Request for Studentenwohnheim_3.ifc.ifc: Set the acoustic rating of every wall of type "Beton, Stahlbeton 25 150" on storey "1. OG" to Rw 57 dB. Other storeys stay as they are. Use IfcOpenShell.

First a look at what the model holds.

```python
import ifcopenshell
import ifcopenshell.util.element

model = ifcopenshell.open("Studentenwohnheim_3.ifc.ifc")
print(model.schema)
storey = next(s for s in model.by_type("IfcBuildingStorey") if s.Name == "1. OG")
walls = [e for e in ifcopenshell.util.element.get_decomposition(storey) if e.is_a("IfcWall")]
seen = {}
for e in walls:
    element_type = ifcopenshell.util.element.get_type(e)
    key = (element_type.Name if element_type != e and element_type else None, ifcopenshell.util.element.get_pset(e, "Pset_WallCommon", "AcousticRating"))
    seen[key] = seen.get(key, 0) + 1
for (name, value), count in sorted(seen.items(), key=str):
    print(count, "x", name, "|", value)
```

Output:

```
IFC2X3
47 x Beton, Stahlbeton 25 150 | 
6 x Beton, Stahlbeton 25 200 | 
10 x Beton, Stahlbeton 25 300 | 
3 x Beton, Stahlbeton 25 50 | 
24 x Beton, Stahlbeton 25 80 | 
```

```python
import ifcopenshell
import ifcopenshell.api.pset
import ifcopenshell.util.element

model = ifcopenshell.open("Studentenwohnheim_3.ifc.ifc")

storey = next(s for s in model.by_type("IfcBuildingStorey") if s.Name == "1. OG")
walls = [e for e in ifcopenshell.util.element.get_decomposition(storey) if e.is_a("IfcWall")]

count = 0
for e in walls:
    element_type = ifcopenshell.util.element.get_type(e)
    if element_type in (None, e) or element_type.Name != "Beton, Stahlbeton 25 150":
        continue
    # add_pset returns the element's existing set when there is one.
    pset = ifcopenshell.api.pset.add_pset(model, product=e, name="Pset_WallCommon")
    ifcopenshell.api.pset.edit_pset(model, pset=pset, properties={"AcousticRating": "Rw 57 dB"})
    count += 1

print(count, "walls updated")

model.write("Studentenwohnheim_3.ifc_updated.ifc")
```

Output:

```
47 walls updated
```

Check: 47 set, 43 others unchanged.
